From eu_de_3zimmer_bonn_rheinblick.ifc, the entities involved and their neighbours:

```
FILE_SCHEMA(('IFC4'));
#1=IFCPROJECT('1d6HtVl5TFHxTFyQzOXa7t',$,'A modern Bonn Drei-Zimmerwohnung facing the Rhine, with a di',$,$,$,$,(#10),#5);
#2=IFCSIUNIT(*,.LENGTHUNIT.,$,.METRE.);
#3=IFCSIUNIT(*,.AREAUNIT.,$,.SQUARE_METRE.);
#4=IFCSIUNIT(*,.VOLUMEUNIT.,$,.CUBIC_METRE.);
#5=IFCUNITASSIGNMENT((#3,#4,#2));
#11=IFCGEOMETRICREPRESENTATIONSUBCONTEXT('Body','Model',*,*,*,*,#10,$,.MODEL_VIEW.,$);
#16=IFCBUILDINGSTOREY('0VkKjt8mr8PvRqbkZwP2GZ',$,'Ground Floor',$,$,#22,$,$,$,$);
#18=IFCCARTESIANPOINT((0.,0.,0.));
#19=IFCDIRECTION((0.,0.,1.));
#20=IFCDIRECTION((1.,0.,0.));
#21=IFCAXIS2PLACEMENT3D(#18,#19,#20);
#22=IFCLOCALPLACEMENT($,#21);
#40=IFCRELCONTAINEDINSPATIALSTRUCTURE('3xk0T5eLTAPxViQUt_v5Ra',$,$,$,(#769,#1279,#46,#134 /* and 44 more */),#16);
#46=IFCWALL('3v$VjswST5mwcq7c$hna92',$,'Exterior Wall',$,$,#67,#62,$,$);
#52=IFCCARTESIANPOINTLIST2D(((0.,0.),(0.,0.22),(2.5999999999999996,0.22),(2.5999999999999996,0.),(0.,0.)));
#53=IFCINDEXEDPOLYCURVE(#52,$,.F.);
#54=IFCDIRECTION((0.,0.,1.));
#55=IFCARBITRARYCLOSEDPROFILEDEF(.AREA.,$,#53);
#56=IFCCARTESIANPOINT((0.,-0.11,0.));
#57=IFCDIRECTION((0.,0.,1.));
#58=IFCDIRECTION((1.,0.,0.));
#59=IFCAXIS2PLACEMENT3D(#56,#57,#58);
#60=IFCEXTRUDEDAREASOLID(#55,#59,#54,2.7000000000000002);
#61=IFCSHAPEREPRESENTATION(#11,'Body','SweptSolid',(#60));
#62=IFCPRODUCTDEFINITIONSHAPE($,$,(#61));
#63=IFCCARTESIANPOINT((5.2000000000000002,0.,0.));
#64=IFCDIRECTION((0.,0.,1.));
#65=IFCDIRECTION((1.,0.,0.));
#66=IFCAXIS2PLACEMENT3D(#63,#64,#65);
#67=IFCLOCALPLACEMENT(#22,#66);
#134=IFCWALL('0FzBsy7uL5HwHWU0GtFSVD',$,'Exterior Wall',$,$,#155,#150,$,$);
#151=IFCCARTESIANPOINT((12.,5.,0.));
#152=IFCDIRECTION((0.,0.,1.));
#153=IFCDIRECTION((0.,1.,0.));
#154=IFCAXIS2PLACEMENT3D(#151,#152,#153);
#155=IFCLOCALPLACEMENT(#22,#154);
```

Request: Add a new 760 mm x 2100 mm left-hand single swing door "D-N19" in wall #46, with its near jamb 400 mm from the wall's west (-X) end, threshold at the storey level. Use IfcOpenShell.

```python
import numpy as np
import ifcopenshell
import ifcopenshell.api.feature
import ifcopenshell.api.geometry
import ifcopenshell.api.root
import ifcopenshell.api.spatial
import ifcopenshell.geom
import ifcopenshell.util.element
import ifcopenshell.util.placement
import ifcopenshell.util.representation
import ifcopenshell.util.shape
import ifcopenshell.util.unit

model = ifcopenshell.open("eu_de_3zimmer_bonn_rheinblick.ifc")
unit_scale = ifcopenshell.util.unit.calculate_unit_scale(model)
settings = ifcopenshell.geom.settings()


def volume(element):
    """Net volume in cubic metres, openings subtracted."""
    shape = ifcopenshell.geom.create_shape(settings, element)
    return ifcopenshell.util.shape.get_volume(shape.geometry)


wall = model.by_guid("3v$VjswST5mwcq7c$hna92")
storey = ifcopenshell.util.element.get_container(wall, ifc_class="IfcBuildingStorey")
context = ifcopenshell.util.representation.get_context(model, "Model", "Body", "MODEL_VIEW")
before = volume(wall)

width, height, from_end, sill = 0.76, 2.1, 0.4, 0.0  # metres

# The wall runs along its own X axis, and the end named is its -X end.
wall_shape = ifcopenshell.geom.create_shape(settings, wall)
x, y, z = ifcopenshell.util.shape.get_vertices(wall_shape.geometry).T
start = x.min() + from_end
face, thickness = float(y.min()), float(y.max() - y.min())
wall_matrix = ifcopenshell.util.placement.get_local_placement(wall.ObjectPlacement)
level = ifcopenshell.util.placement.get_local_placement(storey.ObjectPlacement)[2, 3]


def in_wall(x, y):
    """Placement at x, y metres in the wall's axes, at sill height."""
    matrix = wall_matrix.copy()
    matrix[:, 3] = wall_matrix @ np.array([x / unit_scale, y / unit_scale, 0.0, 1.0])
    matrix[2, 3] = level + sill / unit_scale
    return matrix


# Opening: a box that overshoots both wall faces by 50 mm.
opening = ifcopenshell.api.root.create_entity(model, ifc_class="IfcOpeningElement", predefined_type="OPENING")
box = ifcopenshell.api.geometry.add_wall_representation(
    model, context=context, length=width, height=height, thickness=thickness + 0.1
)
ifcopenshell.api.geometry.assign_representation(model, product=opening, representation=box)
ifcopenshell.api.geometry.edit_object_placement(model, product=opening, matrix=in_wall(start, face - 0.05), is_si=False)
ifcopenshell.api.feature.add_feature(model, feature=opening, element=wall)

door = ifcopenshell.api.root.create_entity(model, ifc_class="IfcDoor", name="D-N19", predefined_type="DOOR")
door.OverallWidth, door.OverallHeight = width / unit_scale, height / unit_scale
door.OperationType = "SINGLE_SWING_LEFT"
body = ifcopenshell.api.geometry.add_door_representation(
    model,
    context=context,
    overall_width=door.OverallWidth,
    overall_height=door.OverallHeight,
    operation_type="SINGLE_SWING_LEFT",
    lining_properties={"LiningDepth": thickness / unit_scale, "ThresholdDepth": thickness / unit_scale},
)
ifcopenshell.api.geometry.assign_representation(model, product=door, representation=body)
ifcopenshell.api.spatial.assign_container(model, products=[door], relating_structure=storey)
ifcopenshell.api.feature.add_filling(model, opening=opening, element=door)

# The lining spans the wall, so the door starts at the wall face.
ifcopenshell.api.geometry.edit_object_placement(model, product=door, matrix=in_wall(start, face), is_si=False)

after = volume(wall)

print(f"wall volume {before:.3f} -> {after:.3f} m3")

model.write("eu_de_3zimmer_bonn_rheinblick_v2.ifc")
```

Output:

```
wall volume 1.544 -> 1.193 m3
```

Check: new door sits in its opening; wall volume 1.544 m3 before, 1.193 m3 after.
